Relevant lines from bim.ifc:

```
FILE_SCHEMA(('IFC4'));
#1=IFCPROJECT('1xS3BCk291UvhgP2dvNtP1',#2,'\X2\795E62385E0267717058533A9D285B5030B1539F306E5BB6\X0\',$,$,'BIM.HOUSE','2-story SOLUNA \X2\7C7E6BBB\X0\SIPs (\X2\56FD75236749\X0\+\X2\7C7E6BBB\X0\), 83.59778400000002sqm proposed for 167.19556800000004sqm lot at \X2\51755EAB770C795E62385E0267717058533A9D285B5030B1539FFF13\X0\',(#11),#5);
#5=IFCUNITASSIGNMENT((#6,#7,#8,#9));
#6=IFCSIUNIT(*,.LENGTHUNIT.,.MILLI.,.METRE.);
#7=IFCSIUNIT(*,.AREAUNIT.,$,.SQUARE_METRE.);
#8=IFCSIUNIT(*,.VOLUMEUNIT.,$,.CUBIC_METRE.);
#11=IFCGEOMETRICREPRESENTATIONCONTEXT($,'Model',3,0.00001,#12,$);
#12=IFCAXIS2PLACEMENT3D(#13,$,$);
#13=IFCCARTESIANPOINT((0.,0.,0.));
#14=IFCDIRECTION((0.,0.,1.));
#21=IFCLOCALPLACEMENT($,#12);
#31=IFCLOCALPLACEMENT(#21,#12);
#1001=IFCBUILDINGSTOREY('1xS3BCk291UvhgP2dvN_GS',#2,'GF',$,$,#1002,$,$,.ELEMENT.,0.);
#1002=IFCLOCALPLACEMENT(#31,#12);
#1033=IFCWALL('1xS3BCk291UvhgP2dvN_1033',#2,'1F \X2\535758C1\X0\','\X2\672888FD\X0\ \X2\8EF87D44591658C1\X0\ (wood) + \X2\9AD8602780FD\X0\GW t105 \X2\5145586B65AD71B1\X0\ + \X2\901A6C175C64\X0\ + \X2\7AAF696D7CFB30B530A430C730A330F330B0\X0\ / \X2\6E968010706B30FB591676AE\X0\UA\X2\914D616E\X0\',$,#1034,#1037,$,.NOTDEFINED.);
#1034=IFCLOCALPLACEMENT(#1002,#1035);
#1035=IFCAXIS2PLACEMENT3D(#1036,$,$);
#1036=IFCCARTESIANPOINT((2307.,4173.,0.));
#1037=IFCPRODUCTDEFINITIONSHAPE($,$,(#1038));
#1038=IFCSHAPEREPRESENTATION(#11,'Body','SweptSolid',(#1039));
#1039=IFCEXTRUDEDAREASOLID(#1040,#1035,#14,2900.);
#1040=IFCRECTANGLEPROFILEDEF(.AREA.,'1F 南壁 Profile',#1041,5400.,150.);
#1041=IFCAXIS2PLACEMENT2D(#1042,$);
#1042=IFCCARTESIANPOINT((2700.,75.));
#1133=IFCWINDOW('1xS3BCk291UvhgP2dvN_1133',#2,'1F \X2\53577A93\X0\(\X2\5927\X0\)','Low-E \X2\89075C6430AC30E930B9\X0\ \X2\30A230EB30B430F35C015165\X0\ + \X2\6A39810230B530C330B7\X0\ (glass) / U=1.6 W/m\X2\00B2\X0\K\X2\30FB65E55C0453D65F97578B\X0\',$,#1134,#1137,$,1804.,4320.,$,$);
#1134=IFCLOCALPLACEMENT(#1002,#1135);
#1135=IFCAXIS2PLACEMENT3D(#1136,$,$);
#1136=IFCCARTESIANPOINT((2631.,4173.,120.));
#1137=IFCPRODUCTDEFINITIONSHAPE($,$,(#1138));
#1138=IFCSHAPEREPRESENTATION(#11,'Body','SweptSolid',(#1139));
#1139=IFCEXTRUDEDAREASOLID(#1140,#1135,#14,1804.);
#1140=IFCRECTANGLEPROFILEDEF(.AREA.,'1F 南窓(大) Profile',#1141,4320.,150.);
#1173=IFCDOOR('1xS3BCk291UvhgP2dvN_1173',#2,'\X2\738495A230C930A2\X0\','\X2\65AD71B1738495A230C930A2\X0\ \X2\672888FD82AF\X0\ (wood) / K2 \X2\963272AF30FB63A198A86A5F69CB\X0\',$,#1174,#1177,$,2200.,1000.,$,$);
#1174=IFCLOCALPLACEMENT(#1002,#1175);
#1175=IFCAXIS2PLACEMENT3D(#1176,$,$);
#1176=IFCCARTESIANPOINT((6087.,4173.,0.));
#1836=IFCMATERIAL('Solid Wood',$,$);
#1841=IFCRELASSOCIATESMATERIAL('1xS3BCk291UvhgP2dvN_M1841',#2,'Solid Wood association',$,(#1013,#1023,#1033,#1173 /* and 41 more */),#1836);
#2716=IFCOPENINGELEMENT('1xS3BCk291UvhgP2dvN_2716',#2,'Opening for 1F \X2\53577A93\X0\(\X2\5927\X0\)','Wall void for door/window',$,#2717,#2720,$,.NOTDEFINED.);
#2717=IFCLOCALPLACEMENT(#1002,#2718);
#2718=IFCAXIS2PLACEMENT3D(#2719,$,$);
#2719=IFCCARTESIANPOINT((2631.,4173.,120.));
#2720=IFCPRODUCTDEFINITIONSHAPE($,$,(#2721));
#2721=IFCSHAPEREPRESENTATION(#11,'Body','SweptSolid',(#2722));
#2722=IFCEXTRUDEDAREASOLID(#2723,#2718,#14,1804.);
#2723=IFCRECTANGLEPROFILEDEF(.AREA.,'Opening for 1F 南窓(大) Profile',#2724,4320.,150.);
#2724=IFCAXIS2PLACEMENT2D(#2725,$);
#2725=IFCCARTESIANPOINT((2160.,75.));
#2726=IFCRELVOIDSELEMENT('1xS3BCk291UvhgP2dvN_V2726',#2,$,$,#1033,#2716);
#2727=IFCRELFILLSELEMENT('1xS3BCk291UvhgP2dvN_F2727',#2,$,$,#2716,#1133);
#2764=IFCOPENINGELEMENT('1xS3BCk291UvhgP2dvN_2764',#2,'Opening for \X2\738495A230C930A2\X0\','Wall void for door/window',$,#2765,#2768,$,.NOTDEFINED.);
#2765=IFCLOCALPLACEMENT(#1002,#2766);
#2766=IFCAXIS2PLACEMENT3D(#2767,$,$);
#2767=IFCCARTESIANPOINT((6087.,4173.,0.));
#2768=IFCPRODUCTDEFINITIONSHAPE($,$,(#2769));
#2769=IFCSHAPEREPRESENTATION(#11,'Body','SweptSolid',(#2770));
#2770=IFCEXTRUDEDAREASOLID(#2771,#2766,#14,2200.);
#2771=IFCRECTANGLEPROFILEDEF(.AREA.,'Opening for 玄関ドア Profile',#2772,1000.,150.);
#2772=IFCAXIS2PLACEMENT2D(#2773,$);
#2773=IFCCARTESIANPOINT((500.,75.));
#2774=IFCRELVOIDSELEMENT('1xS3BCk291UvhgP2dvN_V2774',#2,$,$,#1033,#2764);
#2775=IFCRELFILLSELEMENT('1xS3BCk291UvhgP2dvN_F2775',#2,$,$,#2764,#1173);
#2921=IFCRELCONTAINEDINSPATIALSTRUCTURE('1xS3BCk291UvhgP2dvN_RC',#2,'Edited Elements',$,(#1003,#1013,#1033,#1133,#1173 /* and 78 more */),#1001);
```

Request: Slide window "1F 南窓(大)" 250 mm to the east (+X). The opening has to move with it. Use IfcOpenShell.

```python
import ifcopenshell
import ifcopenshell.api.geometry
import ifcopenshell.util.placement

model = ifcopenshell.open("bim.ifc")

window = model.by_guid("1xS3BCk291UvhgP2dvN_1133")
opening = window.FillsVoids[0].RelatingOpeningElement
wall = opening.VoidsElements[0].RelatingBuildingElement

wall_matrix = ifcopenshell.util.placement.get_local_placement(wall.ObjectPlacement)
shift = wall_matrix[:3, 0] * 250.0
before = ifcopenshell.util.placement.get_local_placement(window.ObjectPlacement)[:3, 3].copy()

# The window is not placed relative to its opening, so move both.
for product in (opening, window):
    matrix = ifcopenshell.util.placement.get_local_placement(product.ObjectPlacement)
    matrix[:3, 3] += shift
    ifcopenshell.api.geometry.edit_object_placement(model, product=product, matrix=matrix, is_si=False)

after = ifcopenshell.util.placement.get_local_placement(window.ObjectPlacement)[:3, 3]
print("window moved by", (after - before).round(3) + 0.0)

model.write("bim_v2.ifc")
```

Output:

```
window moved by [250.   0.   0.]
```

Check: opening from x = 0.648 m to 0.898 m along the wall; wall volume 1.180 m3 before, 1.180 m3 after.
